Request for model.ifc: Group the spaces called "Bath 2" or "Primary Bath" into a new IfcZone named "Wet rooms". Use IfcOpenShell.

First a look at what the model holds.

```python
import ifcopenshell

model = ifcopenshell.open("model.ifc")
print(model.schema)
seen = {}
for space in model.by_type("IfcSpace"):
    seen[space.LongName] = seen.get(space.LongName, 0) + 1
for name, count in sorted(seen.items(), key=str):
    print(count, "x", name)
print("zones:", [z.Name for z in model.by_type("IfcZone")][:20])
```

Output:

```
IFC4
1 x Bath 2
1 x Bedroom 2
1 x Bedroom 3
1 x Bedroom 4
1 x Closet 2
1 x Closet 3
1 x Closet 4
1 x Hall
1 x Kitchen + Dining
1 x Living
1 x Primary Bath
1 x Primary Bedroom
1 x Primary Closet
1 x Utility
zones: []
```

```python
import ifcopenshell
import ifcopenshell.api.group
import ifcopenshell.api.root

model = ifcopenshell.open("model.ifc")

names = {"Bath 2", "Primary Bath"}
spaces = [s for s in model.by_type("IfcSpace") if s.LongName in names]

zone = ifcopenshell.api.root.create_entity(model, ifc_class="IfcZone", name="Wet rooms")
ifcopenshell.api.group.assign_group(model, products=spaces, group=zone)
print(len(spaces), "spaces in", zone.Name)

model.write("model_edited.ifc")
```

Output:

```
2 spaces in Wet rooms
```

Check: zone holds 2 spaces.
